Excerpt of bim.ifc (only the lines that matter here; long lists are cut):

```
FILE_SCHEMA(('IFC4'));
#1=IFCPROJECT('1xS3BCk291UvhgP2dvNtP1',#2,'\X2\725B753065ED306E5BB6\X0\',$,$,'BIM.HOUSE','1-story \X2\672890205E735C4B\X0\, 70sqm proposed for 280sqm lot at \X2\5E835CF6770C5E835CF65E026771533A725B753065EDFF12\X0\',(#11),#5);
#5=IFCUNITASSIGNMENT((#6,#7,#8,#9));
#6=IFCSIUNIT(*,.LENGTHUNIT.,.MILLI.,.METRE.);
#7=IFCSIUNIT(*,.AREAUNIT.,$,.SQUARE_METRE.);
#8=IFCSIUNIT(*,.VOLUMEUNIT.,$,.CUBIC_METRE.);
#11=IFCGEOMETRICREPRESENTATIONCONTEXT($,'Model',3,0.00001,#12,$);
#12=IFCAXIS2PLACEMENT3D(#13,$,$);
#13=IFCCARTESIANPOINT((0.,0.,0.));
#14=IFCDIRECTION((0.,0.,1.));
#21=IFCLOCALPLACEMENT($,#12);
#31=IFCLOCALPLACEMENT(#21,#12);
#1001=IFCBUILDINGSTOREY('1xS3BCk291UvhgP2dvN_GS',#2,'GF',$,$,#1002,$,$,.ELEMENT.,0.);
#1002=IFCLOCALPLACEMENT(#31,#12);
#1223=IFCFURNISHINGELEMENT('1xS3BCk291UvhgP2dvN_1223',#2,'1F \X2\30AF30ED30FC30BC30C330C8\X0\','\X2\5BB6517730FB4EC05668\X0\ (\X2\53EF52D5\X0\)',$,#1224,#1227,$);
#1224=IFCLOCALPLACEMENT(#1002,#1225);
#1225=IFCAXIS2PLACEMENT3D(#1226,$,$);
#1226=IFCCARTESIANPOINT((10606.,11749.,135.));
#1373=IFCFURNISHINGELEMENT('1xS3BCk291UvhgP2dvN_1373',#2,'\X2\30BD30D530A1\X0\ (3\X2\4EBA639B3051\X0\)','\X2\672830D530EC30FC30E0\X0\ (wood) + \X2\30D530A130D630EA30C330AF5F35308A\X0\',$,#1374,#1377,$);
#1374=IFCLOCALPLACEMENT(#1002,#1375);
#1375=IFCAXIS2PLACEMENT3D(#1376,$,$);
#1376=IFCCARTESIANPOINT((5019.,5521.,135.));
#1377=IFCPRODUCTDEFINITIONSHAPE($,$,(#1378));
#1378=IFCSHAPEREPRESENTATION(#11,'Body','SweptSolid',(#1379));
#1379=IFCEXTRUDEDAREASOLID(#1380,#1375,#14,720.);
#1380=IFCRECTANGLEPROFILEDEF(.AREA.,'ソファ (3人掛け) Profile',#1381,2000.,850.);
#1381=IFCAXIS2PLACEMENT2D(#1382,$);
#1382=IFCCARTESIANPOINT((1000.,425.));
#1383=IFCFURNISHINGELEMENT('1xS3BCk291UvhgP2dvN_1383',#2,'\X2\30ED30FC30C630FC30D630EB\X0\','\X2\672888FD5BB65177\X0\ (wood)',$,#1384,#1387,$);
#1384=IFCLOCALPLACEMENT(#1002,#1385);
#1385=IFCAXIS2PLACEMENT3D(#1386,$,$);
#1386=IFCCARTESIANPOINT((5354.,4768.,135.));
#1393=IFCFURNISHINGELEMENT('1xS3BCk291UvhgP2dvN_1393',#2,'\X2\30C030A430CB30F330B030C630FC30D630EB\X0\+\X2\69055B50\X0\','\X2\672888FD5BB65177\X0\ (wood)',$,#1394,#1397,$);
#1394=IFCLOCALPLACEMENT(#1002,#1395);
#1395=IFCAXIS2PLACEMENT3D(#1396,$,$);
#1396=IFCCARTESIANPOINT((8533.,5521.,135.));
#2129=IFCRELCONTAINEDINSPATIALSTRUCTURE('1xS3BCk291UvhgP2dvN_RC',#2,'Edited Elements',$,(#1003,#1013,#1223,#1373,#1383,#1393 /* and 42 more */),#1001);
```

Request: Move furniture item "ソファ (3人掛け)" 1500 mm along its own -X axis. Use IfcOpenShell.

```python
import ifcopenshell
import ifcopenshell.api.geometry
import ifcopenshell.util.placement
import ifcopenshell.util.unit

model = ifcopenshell.open("bim.ifc")
unit_scale = ifcopenshell.util.unit.calculate_unit_scale(model)

item = model.by_guid("1xS3BCk291UvhgP2dvN_1373")
matrix = ifcopenshell.util.placement.get_local_placement(item.ObjectPlacement)
matrix[:3, 3] -= matrix[:3, 0] * 1.5 / unit_scale
ifcopenshell.api.geometry.edit_object_placement(model, product=item, matrix=matrix, is_si=False)

print(ifcopenshell.util.placement.get_local_placement(item.ObjectPlacement).round(3) + 0.0)

model.write("bim_updated.ifc")
```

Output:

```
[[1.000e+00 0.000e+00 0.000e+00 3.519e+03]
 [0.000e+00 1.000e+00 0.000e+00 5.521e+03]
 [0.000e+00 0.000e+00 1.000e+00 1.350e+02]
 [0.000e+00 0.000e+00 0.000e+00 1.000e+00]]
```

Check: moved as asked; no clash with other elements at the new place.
